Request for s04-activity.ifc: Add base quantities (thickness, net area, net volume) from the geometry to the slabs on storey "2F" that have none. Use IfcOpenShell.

First a look at what the model holds.

```python
import ifcopenshell
import ifcopenshell.util.element
import ifcopenshell.util.unit

model = ifcopenshell.open("s04-activity.ifc")
print(model.schema)
for unit_type in ("LENGTHUNIT", "AREAUNIT", "VOLUMEUNIT"):
    print(unit_type, ifcopenshell.util.unit.calculate_unit_scale(model, unit_type))
storey = next(s for s in model.by_type("IfcBuildingStorey") if s.Name == "2F")
slabs = [e for e in ifcopenshell.util.element.get_decomposition(storey) if e.is_a("IfcSlab")]
for e in sorted(slabs, key=lambda e: e.id()):
    print(e.id(), e.is_a(), e.Name, list(ifcopenshell.util.element.get_psets(e, qtos_only=True)), sep=" | ")
```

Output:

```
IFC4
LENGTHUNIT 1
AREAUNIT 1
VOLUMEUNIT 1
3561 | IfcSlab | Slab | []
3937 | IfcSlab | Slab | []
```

```python
import ifcopenshell
import ifcopenshell.api.pset
import ifcopenshell.geom
import ifcopenshell.util.element
import ifcopenshell.util.shape
import ifcopenshell.util.unit

model = ifcopenshell.open("s04-activity.ifc")
unit_scale = ifcopenshell.util.unit.calculate_unit_scale(model)
area_scale = ifcopenshell.util.unit.calculate_unit_scale(model, "AREAUNIT")
volume_scale = ifcopenshell.util.unit.calculate_unit_scale(model, "VOLUMEUNIT")
settings = ifcopenshell.geom.settings()

storey = next(s for s in model.by_type("IfcBuildingStorey") if s.Name == "2F")
slabs = [e for e in ifcopenshell.util.element.get_decomposition(storey) if e.is_a("IfcSlab")]

for e in sorted(slabs, key=lambda e: e.id()):
    if ifcopenshell.util.element.get_psets(e, qtos_only=True, should_inherit=False):
        continue
    # Geometry comes back in metres, in the element's own axes.
    shape = ifcopenshell.geom.create_shape(settings, e)
    values = {
        "Width": ifcopenshell.util.shape.get_z(shape.geometry) / unit_scale,
        "NetArea": ifcopenshell.util.shape.get_footprint_area(shape.geometry) / area_scale,
        "NetVolume": ifcopenshell.util.shape.get_volume(shape.geometry) / volume_scale,
    }
    qto = ifcopenshell.api.pset.add_qto(model, product=e, name="Qto_SlabBaseQuantities")
    ifcopenshell.api.pset.edit_qto(model, qto=qto, properties=values)
    print(e.id(), {k: round(v, 3) for k, v in values.items()})

model.write("s04-activity-out.ifc")
```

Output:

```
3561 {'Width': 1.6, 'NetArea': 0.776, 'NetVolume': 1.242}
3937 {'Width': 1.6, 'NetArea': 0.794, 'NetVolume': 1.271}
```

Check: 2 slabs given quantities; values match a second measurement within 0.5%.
